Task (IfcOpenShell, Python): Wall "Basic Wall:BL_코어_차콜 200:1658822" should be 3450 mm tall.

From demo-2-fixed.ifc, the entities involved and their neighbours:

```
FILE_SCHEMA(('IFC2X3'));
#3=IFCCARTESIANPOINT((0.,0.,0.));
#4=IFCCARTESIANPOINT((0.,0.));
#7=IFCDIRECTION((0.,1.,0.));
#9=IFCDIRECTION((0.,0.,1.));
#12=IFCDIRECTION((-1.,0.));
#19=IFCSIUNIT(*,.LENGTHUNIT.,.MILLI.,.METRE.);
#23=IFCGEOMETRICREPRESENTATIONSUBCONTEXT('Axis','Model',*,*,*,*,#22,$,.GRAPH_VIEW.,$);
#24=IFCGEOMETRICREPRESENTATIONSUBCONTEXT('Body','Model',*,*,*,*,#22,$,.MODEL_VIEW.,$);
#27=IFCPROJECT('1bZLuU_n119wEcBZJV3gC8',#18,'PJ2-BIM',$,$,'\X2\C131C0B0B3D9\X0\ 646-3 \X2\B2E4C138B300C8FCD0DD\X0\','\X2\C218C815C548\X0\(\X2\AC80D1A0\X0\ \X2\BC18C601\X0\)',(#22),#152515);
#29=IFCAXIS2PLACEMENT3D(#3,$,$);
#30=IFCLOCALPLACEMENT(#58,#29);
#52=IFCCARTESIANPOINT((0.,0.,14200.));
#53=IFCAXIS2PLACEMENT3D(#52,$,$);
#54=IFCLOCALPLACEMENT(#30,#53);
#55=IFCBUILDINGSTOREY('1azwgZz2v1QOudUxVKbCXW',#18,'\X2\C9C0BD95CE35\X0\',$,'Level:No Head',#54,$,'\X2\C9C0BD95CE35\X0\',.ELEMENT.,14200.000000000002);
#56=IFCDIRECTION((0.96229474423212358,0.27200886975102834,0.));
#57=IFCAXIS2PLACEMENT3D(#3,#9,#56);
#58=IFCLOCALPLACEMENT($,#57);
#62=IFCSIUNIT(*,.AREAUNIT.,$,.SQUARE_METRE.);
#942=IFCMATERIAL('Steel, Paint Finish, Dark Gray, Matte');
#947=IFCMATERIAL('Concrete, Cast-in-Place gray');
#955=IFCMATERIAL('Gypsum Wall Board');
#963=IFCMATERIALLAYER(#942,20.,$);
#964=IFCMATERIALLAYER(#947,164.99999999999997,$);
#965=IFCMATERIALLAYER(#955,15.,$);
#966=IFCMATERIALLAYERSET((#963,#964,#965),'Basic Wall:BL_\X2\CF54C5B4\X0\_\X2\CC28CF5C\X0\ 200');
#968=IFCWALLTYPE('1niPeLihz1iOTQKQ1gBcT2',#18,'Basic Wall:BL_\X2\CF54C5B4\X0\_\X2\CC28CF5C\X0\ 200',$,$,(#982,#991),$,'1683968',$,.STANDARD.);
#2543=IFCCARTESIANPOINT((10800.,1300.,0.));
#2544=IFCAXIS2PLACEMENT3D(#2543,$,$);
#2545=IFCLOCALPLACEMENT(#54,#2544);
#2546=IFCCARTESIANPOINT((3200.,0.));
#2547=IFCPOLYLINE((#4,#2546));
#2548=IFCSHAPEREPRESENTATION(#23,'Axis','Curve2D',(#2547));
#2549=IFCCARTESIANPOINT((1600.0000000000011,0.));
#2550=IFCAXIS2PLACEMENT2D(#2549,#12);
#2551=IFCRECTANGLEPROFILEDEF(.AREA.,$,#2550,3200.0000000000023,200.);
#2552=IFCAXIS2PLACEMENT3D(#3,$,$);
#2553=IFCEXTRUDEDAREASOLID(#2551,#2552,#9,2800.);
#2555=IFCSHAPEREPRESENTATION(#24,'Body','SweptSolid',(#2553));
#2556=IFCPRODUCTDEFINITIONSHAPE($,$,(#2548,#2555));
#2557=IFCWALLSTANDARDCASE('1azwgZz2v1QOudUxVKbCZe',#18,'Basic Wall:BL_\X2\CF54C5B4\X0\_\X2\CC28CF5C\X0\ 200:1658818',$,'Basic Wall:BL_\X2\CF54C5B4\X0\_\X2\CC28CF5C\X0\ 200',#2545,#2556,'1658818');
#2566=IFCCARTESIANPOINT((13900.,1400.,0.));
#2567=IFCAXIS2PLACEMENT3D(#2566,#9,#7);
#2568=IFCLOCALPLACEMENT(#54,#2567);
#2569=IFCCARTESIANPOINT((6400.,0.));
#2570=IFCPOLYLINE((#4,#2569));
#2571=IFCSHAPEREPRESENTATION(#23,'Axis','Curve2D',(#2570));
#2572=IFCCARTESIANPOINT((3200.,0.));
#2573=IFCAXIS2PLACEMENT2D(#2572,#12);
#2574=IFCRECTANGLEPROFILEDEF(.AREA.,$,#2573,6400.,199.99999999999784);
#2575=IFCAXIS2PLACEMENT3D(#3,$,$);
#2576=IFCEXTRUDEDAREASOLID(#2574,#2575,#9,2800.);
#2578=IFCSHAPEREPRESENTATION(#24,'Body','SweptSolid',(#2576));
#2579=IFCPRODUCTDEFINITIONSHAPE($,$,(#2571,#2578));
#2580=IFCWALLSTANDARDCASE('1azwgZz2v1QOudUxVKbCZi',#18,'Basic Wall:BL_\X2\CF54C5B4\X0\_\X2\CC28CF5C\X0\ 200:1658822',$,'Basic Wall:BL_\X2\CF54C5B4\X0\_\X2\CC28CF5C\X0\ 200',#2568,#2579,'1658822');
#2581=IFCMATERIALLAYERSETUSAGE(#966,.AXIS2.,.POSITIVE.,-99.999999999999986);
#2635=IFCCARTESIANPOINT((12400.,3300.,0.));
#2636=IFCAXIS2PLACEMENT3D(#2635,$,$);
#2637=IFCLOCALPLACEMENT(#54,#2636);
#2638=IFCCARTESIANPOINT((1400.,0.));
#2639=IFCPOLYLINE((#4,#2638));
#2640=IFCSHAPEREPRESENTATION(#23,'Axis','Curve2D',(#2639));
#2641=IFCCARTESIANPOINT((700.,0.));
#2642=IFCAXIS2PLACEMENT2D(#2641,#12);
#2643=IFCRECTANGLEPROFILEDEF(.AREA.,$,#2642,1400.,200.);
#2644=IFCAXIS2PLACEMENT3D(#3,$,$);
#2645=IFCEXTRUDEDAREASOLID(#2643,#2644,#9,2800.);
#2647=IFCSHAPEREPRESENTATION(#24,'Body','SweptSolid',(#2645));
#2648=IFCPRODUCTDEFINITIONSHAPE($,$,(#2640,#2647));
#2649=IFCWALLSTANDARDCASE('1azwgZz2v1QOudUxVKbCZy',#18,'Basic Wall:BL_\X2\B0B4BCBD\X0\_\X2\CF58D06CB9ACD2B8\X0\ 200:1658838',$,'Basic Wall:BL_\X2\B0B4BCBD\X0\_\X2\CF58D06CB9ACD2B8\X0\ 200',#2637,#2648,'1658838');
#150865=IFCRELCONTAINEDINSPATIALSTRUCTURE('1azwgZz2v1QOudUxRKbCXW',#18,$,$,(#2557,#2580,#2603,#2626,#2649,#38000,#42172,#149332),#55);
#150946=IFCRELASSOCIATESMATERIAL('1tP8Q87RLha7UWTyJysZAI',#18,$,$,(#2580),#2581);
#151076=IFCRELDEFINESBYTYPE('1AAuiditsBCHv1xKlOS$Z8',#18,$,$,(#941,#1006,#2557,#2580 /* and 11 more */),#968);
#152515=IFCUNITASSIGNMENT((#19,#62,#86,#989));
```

```python
import ifcopenshell
import ifcopenshell.geom
import ifcopenshell.util.representation
import ifcopenshell.util.shape

model = ifcopenshell.open("demo-2-fixed.ifc")
settings = ifcopenshell.geom.settings()


def volume(element):
    """Net volume in cubic metres, openings subtracted."""
    shape = ifcopenshell.geom.create_shape(settings, element)
    return ifcopenshell.util.shape.get_volume(shape.geometry)


wall = model.by_guid("1azwgZz2v1QOudUxVKbCZi")
before = volume(wall)

body = ifcopenshell.util.representation.get_representation(wall, "Model", "Body")
solid = body.Items[0]
old_height = solid.Depth
solid.Depth = 3450.0
after = volume(wall)

print(f"height {old_height:g} -> {solid.Depth:g}, volume {before:.3f} -> {after:.3f} m3")

model.write("demo-2-fixed-out.ifc")
```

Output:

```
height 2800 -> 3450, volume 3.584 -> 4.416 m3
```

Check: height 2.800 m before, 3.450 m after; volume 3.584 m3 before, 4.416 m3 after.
